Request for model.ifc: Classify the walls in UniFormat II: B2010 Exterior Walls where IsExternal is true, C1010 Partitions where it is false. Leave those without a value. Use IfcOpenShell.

First a look at what the model holds.

```python
import ifcopenshell
import ifcopenshell.util.element

model = ifcopenshell.open("model.ifc")
print(model.schema)
print("classifications:", [c.Name for c in model.by_type("IfcClassification")])
values = [ifcopenshell.util.element.get_pset(e, "Pset_WallCommon", "IsExternal") for e in model.by_type("IfcWall")]
for value in (True, False, None):
    print("IsExternal", value, values.count(value))
```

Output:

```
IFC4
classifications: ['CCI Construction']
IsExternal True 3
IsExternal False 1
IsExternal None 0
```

```python
import ifcopenshell
import ifcopenshell.api.classification
import ifcopenshell.util.element

model = ifcopenshell.open("model.ifc")

system = ifcopenshell.api.classification.add_classification(model, classification="UniFormat II")

walls = model.by_type("IfcWall")
external = {e: ifcopenshell.util.element.get_pset(e, "Pset_WallCommon", "IsExternal") for e in walls}
for flag, code, name in ((True, "B2010", "Exterior Walls"), (False, "C1010", "Partitions")):
    products = [e for e in walls if external[e] is flag]
    ifcopenshell.api.classification.add_reference(
        model, products=products, classification=system, identification=code, name=name
    )
    print(code, len(products))

model.write("model_v2.ifc")
```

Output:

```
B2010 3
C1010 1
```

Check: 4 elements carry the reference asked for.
